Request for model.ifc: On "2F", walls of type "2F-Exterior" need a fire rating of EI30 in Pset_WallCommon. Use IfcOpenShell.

First a look at what the model holds.

```python
import ifcopenshell
import ifcopenshell.util.element

model = ifcopenshell.open("model.ifc")
print(model.schema)
storey = next(s for s in model.by_type("IfcBuildingStorey") if s.Name == "2F")
walls = [e for e in ifcopenshell.util.element.get_decomposition(storey) if e.is_a("IfcWall")]
seen = {}
for e in walls:
    element_type = ifcopenshell.util.element.get_type(e)
    key = (element_type.Name if element_type != e and element_type else None, ifcopenshell.util.element.get_pset(e, "Pset_WallCommon", "FireRating"))
    seen[key] = seen.get(key, 0) + 1
for (name, value), count in sorted(seen.items(), key=str):
    print(count, "x", name, "|", value)
```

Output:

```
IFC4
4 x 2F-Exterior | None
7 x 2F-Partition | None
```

```python
import ifcopenshell
import ifcopenshell.api.pset
import ifcopenshell.util.element

model = ifcopenshell.open("model.ifc")

storey = next(s for s in model.by_type("IfcBuildingStorey") if s.Name == "2F")
walls = [e for e in ifcopenshell.util.element.get_decomposition(storey) if e.is_a("IfcWall")]

count = 0
for e in walls:
    element_type = ifcopenshell.util.element.get_type(e)
    if element_type in (None, e) or element_type.Name != "2F-Exterior":
        continue
    # add_pset returns the element's existing set when there is one.
    pset = ifcopenshell.api.pset.add_pset(model, product=e, name="Pset_WallCommon")
    ifcopenshell.api.pset.edit_pset(model, pset=pset, properties={"FireRating": "EI30"})
    count += 1

print(count, "walls updated")

model.write("model_updated.ifc")
```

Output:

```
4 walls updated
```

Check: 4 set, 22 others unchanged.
